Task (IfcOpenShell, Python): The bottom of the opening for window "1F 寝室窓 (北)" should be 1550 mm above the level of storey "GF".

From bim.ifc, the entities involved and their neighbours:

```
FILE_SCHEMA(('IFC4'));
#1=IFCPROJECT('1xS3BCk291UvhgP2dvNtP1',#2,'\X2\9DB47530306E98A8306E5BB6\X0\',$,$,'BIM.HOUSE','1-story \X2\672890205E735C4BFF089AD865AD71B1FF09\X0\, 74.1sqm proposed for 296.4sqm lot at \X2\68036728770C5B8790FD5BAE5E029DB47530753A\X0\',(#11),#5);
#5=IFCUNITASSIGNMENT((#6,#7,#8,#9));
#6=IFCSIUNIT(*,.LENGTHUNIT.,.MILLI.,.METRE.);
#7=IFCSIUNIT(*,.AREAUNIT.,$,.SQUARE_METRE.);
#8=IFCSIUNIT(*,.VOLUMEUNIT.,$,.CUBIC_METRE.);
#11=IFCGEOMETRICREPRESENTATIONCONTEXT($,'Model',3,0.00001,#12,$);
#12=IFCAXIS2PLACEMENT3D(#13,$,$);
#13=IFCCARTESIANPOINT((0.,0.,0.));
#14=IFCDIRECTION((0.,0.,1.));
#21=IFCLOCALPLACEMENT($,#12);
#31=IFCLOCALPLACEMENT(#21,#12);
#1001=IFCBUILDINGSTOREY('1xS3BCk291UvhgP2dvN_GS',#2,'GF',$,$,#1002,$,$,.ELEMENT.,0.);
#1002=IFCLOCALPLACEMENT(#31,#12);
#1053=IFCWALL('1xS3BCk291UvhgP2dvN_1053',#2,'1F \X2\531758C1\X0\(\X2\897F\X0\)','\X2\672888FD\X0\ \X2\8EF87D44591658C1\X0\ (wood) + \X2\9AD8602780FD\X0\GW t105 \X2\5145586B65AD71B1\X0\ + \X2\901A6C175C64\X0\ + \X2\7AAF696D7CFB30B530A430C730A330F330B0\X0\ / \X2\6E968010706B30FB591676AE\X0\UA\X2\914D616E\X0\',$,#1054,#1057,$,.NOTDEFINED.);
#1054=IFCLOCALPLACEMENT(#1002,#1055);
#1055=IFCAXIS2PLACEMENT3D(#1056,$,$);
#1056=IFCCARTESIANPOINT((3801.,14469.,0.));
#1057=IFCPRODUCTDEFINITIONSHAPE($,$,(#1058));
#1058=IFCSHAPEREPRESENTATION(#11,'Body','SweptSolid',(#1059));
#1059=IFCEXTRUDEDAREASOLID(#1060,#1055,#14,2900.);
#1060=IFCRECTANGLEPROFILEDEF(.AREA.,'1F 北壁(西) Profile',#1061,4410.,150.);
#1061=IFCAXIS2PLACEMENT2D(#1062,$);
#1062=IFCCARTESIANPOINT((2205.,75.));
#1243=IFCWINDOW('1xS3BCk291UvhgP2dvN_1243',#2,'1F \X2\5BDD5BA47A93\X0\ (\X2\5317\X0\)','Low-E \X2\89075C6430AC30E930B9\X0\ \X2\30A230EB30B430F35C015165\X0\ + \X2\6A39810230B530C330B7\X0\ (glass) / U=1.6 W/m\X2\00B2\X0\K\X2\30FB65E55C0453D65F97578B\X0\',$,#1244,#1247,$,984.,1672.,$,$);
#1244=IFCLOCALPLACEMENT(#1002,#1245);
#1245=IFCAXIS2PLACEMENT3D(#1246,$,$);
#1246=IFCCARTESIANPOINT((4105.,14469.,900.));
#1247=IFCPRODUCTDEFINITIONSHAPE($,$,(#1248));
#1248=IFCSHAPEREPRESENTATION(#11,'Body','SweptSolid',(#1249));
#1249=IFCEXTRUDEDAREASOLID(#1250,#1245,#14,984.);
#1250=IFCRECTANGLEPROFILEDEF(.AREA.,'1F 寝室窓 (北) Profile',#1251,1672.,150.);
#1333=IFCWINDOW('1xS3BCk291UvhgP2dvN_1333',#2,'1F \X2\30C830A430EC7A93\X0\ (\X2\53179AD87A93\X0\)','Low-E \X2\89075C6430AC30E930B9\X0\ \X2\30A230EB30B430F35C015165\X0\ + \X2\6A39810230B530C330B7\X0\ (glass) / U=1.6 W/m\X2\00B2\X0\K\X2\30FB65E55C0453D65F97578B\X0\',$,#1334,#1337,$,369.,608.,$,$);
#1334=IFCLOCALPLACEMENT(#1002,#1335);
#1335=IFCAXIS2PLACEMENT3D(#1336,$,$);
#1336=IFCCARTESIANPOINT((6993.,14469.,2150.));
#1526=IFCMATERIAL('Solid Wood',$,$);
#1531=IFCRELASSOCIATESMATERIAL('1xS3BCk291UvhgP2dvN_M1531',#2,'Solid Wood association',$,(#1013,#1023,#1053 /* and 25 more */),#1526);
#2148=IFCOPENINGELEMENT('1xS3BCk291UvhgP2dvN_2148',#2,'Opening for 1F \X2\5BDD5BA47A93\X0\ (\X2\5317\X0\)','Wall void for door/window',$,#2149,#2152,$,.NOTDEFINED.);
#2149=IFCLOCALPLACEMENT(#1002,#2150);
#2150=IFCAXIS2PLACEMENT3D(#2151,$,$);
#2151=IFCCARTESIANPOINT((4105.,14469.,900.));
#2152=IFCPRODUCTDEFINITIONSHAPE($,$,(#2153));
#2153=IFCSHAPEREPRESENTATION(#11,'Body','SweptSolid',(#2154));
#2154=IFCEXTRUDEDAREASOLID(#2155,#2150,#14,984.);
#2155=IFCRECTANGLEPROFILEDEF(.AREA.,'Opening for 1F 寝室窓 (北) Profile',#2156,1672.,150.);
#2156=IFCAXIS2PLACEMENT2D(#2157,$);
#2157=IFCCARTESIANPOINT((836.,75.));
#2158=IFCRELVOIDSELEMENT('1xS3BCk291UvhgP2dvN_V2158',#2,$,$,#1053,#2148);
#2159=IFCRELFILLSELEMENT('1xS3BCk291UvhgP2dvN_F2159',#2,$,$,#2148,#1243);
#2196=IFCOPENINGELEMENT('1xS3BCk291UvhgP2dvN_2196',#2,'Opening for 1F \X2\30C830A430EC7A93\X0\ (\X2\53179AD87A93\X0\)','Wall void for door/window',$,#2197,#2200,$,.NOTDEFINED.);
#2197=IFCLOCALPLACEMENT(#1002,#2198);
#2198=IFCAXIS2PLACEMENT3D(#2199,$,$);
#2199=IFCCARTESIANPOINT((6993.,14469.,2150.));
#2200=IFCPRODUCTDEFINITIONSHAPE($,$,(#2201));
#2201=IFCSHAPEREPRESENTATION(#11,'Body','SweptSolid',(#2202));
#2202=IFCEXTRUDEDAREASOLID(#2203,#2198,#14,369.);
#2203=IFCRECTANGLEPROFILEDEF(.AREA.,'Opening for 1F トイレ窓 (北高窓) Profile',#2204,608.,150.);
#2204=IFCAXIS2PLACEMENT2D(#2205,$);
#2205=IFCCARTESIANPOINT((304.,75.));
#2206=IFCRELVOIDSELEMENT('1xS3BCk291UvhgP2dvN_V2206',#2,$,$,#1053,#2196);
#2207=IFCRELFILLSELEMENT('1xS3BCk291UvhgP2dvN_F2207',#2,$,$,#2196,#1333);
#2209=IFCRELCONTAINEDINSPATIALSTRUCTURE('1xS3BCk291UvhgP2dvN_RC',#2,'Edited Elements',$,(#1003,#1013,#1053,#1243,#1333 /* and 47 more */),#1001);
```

```python
import numpy as np
import ifcopenshell
import ifcopenshell.api.geometry
import ifcopenshell.geom
import ifcopenshell.util.element
import ifcopenshell.util.placement
import ifcopenshell.util.shape
import ifcopenshell.util.unit

model = ifcopenshell.open("bim.ifc")
unit_scale = ifcopenshell.util.unit.calculate_unit_scale(model)

window = model.by_guid("1xS3BCk291UvhgP2dvN_1243")
opening = window.FillsVoids[0].RelatingOpeningElement
storey = ifcopenshell.util.element.get_container(window, ifc_class="IfcBuildingStorey")
level = ifcopenshell.util.placement.get_local_placement(storey.ObjectPlacement)[2, 3]

# The opening's origin need not be at the sill, so measure its lowest point.
shape = ifcopenshell.geom.create_shape(ifcopenshell.geom.settings(), opening)
bottom = ifcopenshell.util.shape.get_shape_bottom_elevation(shape, shape.geometry) / unit_scale
dz = level + 1.55 / unit_scale - bottom

shift = np.array([0.0, 0.0, dz])
# The window is not placed relative to its opening, so move both.
for product in (opening, window):
    matrix = ifcopenshell.util.placement.get_local_placement(product.ObjectPlacement)
    matrix[:3, 3] += shift
    ifcopenshell.api.geometry.edit_object_placement(model, product=product, matrix=matrix, is_si=False)

print(f"moved by {dz * unit_scale:+.3f} m")

model.write("bim_updated.ifc")
```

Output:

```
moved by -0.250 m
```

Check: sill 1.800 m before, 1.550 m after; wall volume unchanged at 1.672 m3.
